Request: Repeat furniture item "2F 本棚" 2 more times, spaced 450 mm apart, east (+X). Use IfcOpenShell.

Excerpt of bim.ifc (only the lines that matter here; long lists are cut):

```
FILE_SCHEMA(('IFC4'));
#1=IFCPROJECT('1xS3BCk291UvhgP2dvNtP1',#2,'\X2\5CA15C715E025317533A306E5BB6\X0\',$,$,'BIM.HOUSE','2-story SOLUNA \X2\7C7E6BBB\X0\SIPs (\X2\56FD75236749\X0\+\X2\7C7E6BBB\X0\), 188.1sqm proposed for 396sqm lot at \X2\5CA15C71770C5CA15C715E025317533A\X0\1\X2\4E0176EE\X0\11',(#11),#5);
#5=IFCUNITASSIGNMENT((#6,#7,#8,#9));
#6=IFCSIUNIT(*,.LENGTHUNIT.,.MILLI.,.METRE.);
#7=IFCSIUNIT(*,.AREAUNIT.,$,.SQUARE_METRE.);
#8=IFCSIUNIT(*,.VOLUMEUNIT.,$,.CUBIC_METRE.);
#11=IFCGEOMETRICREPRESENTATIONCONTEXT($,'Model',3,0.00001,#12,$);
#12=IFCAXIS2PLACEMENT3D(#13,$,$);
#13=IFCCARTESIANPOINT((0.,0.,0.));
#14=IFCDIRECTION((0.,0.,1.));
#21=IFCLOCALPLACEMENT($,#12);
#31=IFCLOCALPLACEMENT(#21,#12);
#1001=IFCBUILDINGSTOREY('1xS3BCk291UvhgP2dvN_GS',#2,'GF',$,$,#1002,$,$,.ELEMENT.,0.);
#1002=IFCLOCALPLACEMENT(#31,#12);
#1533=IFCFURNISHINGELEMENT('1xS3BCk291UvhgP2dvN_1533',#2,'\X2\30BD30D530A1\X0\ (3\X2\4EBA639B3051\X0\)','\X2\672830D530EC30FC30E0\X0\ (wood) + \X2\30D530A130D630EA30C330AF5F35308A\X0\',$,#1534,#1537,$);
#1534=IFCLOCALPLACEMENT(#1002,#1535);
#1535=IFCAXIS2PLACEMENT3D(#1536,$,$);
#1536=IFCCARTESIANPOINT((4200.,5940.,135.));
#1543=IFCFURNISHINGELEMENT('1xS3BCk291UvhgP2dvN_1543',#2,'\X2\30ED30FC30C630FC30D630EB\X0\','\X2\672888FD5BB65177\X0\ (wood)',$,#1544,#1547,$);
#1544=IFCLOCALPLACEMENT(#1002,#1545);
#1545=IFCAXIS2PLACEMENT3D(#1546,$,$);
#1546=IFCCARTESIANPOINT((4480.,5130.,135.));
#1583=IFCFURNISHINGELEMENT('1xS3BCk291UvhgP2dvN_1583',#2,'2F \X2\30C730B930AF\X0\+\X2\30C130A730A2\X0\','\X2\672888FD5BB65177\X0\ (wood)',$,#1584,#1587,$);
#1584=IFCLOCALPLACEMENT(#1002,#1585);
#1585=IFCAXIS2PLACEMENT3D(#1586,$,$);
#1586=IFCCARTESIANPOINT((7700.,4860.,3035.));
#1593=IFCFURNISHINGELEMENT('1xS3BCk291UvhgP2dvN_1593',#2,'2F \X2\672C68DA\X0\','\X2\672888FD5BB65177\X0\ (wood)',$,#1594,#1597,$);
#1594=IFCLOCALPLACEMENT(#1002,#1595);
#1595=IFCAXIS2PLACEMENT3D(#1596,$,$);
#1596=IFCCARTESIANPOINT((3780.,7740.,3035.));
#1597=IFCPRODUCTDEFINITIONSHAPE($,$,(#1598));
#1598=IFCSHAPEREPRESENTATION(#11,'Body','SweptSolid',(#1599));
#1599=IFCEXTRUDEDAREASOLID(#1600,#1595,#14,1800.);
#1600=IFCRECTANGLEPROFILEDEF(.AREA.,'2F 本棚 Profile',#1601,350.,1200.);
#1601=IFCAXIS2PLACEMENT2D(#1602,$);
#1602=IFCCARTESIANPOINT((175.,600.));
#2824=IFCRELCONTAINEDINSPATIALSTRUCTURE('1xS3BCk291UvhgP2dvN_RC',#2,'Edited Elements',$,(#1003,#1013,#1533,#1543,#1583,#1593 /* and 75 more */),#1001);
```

```python
import numpy as np
import ifcopenshell
import ifcopenshell.api.geometry
import ifcopenshell.api.root
import ifcopenshell.util.element
import ifcopenshell.util.placement
import ifcopenshell.util.unit

model = ifcopenshell.open("bim.ifc")
unit_scale = ifcopenshell.util.unit.calculate_unit_scale(model)


def reuse_history(source, copy):
    """copy_class also copies each property set's owner history, people and application; keep the originals."""
    for rel in copy.IsDefinedBy:
        if rel.is_a("IfcRelDefinesByProperties") and (history := rel.RelatingPropertyDefinition.OwnerHistory):
            rel.RelatingPropertyDefinition.OwnerHistory = source.OwnerHistory
            ifcopenshell.util.element.remove_deep2(model, history)


source = model.by_guid("1xS3BCk291UvhgP2dvN_1593")
base = ifcopenshell.util.placement.get_local_placement(source.ObjectPlacement)
step = np.array([1.0, 0.0, 0.0]) * 0.45 / unit_scale

for i in range(1, 3):
    copy = ifcopenshell.api.root.copy_class(model, product=source)
    copy.Representation = ifcopenshell.util.element.copy_deep(
        model, source.Representation, exclude=["IfcGeometricRepresentationContext", "IfcRepresentationMap"]
    )
    reuse_history(source, copy)
    matrix = base.copy()
    matrix[:3, 3] += i * step
    print("added at", matrix[:3, 3].round(3) + 0.0)
    ifcopenshell.api.geometry.edit_object_placement(model, product=copy, matrix=matrix, is_si=False)

model.write("bim_edited.ifc")
```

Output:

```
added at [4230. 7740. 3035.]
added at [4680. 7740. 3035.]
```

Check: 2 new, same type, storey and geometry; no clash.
